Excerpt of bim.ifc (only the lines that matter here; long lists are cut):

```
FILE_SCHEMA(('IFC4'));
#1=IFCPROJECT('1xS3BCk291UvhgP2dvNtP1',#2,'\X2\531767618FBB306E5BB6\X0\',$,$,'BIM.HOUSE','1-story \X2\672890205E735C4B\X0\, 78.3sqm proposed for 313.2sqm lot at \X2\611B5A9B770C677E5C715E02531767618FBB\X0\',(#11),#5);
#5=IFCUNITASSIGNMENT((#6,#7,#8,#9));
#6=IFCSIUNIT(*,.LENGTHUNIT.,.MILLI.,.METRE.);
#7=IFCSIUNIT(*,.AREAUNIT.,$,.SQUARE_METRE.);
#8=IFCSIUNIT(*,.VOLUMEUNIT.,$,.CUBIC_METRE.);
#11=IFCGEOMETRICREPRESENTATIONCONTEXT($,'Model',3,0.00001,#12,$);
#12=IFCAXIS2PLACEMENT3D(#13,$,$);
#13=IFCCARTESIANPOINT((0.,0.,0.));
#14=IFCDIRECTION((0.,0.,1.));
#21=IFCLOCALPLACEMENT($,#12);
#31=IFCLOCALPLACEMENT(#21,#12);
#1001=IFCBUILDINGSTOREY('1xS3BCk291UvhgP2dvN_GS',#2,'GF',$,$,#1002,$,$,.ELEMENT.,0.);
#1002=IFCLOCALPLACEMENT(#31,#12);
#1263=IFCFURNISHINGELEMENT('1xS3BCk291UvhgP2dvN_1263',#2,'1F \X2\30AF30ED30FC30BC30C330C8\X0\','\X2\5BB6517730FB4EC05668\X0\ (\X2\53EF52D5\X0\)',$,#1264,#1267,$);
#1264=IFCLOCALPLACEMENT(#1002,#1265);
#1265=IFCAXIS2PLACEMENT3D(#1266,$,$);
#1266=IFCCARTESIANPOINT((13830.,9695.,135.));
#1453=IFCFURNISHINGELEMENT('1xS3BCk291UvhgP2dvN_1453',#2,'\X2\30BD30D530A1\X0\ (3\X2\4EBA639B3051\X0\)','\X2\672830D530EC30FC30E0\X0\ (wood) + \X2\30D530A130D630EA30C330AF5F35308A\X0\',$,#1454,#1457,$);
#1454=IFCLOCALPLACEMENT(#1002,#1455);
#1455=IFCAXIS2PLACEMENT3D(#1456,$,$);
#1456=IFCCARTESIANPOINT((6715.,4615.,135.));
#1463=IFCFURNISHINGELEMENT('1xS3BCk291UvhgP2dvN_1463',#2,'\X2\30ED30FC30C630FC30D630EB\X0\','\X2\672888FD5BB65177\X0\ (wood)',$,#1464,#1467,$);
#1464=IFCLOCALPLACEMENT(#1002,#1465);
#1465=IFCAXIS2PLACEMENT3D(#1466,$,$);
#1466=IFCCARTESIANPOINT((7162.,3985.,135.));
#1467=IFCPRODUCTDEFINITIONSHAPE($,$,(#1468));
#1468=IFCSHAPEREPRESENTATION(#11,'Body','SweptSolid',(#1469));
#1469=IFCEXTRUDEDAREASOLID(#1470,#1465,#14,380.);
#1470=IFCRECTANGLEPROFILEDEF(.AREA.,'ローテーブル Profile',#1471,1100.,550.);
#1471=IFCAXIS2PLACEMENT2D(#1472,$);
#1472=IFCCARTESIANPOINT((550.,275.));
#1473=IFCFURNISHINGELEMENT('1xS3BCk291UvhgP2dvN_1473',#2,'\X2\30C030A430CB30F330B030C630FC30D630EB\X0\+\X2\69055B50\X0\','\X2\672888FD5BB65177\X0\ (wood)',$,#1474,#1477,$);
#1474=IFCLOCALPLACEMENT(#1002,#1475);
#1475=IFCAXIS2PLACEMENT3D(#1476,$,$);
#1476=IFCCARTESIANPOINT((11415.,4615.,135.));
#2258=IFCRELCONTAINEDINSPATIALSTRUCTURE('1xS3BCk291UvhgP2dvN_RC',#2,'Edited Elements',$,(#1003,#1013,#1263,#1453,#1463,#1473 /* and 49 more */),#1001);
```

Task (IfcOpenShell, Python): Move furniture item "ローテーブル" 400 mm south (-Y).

```python
import ifcopenshell
import ifcopenshell.api.geometry
import ifcopenshell.util.placement
import ifcopenshell.util.unit

model = ifcopenshell.open("bim.ifc")
unit_scale = ifcopenshell.util.unit.calculate_unit_scale(model)

item = model.by_guid("1xS3BCk291UvhgP2dvN_1463")
matrix = ifcopenshell.util.placement.get_local_placement(item.ObjectPlacement)
matrix[1, 3] -= 0.4 / unit_scale
ifcopenshell.api.geometry.edit_object_placement(model, product=item, matrix=matrix, is_si=False)

print(ifcopenshell.util.placement.get_local_placement(item.ObjectPlacement).round(3) + 0.0)

model.write("bim_rev.ifc")
```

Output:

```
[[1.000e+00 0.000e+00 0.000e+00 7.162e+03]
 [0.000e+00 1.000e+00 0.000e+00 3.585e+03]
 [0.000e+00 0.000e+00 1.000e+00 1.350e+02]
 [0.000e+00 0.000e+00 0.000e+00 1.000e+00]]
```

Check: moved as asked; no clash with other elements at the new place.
